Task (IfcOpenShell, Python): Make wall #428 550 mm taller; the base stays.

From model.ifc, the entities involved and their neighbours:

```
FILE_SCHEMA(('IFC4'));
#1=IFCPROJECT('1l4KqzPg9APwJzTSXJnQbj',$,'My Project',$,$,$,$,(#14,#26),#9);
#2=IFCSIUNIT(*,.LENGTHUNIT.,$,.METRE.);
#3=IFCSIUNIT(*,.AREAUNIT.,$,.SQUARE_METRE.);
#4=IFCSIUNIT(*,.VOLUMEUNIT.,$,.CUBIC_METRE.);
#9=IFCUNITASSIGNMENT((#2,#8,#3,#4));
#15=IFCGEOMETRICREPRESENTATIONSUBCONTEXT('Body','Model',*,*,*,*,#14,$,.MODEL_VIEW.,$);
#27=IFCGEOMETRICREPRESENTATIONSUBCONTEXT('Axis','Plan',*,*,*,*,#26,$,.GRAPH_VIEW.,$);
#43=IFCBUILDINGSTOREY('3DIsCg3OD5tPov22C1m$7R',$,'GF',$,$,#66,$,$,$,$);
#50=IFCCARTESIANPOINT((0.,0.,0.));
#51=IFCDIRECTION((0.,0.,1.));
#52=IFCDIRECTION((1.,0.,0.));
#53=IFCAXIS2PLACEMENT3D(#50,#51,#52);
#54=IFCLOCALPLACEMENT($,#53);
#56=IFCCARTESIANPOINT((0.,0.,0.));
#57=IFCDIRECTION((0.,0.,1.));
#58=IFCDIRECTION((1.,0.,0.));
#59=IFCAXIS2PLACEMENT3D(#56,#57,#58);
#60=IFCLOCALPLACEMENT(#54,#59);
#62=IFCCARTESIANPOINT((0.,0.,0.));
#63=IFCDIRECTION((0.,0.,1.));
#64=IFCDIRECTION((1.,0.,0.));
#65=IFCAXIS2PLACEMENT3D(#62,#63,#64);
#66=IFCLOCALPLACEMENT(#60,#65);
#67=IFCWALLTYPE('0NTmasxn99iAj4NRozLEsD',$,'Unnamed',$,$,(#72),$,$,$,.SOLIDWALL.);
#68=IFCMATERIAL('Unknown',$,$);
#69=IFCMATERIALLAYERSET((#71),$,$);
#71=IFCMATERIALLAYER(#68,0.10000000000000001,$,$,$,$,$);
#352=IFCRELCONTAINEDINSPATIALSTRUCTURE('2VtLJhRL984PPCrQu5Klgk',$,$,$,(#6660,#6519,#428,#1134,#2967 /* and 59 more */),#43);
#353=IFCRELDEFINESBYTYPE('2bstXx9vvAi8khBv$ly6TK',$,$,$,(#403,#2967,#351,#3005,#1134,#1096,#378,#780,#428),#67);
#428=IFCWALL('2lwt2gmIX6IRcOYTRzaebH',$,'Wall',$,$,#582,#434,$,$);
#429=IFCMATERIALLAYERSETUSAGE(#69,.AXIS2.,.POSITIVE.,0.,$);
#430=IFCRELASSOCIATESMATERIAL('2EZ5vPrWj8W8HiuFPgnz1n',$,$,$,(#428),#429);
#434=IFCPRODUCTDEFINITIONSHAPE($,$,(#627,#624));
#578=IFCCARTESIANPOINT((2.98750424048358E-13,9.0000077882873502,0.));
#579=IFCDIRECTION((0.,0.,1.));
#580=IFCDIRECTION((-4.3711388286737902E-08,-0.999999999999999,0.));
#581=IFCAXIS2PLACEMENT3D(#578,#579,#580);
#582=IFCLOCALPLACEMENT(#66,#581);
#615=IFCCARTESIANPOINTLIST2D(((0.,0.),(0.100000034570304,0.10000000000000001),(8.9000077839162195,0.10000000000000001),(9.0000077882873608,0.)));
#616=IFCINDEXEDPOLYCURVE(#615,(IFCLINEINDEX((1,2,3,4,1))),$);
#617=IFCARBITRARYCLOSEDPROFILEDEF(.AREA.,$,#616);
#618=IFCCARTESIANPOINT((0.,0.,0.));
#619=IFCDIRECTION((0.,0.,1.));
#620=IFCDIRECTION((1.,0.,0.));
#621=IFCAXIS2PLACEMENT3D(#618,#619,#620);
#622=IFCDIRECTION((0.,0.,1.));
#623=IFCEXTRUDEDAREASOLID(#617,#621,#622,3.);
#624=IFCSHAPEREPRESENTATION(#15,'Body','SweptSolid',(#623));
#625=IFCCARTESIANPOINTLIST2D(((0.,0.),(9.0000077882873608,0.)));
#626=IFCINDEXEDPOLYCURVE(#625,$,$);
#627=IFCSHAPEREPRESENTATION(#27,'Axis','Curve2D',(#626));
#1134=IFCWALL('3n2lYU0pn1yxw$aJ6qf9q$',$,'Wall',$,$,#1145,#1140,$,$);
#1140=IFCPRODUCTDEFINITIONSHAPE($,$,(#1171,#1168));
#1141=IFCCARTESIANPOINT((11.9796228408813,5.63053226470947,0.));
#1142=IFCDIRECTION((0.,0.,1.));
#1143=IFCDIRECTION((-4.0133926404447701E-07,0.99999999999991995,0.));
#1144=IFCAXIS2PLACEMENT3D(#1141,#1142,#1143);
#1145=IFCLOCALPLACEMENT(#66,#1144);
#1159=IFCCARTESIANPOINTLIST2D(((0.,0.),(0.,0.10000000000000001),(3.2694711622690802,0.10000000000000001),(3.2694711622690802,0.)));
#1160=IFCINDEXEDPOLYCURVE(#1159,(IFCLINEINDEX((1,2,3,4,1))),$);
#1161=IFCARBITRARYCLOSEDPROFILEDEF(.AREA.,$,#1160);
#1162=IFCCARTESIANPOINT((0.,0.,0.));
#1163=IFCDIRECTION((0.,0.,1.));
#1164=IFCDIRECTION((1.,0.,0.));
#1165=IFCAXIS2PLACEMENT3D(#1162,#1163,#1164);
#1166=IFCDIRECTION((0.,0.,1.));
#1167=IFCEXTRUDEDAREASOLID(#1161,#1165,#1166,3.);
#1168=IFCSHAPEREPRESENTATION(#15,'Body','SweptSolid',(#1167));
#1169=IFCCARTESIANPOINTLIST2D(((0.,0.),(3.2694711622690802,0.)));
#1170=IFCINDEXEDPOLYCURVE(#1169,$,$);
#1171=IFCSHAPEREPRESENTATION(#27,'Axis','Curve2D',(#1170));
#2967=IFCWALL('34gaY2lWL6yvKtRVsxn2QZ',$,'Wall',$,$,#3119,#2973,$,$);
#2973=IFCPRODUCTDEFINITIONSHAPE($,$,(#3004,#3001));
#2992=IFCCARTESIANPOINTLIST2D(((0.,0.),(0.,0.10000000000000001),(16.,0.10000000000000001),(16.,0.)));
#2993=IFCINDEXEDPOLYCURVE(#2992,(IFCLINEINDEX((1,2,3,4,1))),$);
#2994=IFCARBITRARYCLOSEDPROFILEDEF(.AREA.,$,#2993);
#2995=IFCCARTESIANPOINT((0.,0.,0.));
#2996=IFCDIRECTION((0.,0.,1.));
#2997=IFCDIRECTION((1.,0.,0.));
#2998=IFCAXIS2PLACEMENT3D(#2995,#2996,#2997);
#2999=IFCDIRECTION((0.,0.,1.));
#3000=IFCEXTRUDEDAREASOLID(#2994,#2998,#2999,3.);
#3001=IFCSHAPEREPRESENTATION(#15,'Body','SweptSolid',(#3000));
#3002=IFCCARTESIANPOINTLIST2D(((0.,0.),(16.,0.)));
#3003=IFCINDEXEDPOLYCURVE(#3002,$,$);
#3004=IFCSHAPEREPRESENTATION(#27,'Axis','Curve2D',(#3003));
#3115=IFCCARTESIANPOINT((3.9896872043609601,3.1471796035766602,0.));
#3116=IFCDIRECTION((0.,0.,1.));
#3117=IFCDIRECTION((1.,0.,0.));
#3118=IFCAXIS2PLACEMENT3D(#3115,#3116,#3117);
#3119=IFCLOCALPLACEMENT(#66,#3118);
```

```python
import ifcopenshell
import ifcopenshell.geom
import ifcopenshell.util.representation
import ifcopenshell.util.shape

model = ifcopenshell.open("model.ifc")
settings = ifcopenshell.geom.settings()


def volume(element):
    """Net volume in cubic metres, openings subtracted."""
    shape = ifcopenshell.geom.create_shape(settings, element)
    return ifcopenshell.util.shape.get_volume(shape.geometry)


wall = model.by_guid("2lwt2gmIX6IRcOYTRzaebH")
before = volume(wall)

body = ifcopenshell.util.representation.get_representation(wall, "Model", "Body")
solid = body.Items[0]
old_height = solid.Depth
solid.Depth += 0.55
after = volume(wall)

print(f"height {old_height:g} -> {solid.Depth:g}, volume {before:.3f} -> {after:.3f} m3")

model.write("model_rev.ifc")
```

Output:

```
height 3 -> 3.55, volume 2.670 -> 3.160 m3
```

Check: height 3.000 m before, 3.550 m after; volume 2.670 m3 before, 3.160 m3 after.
